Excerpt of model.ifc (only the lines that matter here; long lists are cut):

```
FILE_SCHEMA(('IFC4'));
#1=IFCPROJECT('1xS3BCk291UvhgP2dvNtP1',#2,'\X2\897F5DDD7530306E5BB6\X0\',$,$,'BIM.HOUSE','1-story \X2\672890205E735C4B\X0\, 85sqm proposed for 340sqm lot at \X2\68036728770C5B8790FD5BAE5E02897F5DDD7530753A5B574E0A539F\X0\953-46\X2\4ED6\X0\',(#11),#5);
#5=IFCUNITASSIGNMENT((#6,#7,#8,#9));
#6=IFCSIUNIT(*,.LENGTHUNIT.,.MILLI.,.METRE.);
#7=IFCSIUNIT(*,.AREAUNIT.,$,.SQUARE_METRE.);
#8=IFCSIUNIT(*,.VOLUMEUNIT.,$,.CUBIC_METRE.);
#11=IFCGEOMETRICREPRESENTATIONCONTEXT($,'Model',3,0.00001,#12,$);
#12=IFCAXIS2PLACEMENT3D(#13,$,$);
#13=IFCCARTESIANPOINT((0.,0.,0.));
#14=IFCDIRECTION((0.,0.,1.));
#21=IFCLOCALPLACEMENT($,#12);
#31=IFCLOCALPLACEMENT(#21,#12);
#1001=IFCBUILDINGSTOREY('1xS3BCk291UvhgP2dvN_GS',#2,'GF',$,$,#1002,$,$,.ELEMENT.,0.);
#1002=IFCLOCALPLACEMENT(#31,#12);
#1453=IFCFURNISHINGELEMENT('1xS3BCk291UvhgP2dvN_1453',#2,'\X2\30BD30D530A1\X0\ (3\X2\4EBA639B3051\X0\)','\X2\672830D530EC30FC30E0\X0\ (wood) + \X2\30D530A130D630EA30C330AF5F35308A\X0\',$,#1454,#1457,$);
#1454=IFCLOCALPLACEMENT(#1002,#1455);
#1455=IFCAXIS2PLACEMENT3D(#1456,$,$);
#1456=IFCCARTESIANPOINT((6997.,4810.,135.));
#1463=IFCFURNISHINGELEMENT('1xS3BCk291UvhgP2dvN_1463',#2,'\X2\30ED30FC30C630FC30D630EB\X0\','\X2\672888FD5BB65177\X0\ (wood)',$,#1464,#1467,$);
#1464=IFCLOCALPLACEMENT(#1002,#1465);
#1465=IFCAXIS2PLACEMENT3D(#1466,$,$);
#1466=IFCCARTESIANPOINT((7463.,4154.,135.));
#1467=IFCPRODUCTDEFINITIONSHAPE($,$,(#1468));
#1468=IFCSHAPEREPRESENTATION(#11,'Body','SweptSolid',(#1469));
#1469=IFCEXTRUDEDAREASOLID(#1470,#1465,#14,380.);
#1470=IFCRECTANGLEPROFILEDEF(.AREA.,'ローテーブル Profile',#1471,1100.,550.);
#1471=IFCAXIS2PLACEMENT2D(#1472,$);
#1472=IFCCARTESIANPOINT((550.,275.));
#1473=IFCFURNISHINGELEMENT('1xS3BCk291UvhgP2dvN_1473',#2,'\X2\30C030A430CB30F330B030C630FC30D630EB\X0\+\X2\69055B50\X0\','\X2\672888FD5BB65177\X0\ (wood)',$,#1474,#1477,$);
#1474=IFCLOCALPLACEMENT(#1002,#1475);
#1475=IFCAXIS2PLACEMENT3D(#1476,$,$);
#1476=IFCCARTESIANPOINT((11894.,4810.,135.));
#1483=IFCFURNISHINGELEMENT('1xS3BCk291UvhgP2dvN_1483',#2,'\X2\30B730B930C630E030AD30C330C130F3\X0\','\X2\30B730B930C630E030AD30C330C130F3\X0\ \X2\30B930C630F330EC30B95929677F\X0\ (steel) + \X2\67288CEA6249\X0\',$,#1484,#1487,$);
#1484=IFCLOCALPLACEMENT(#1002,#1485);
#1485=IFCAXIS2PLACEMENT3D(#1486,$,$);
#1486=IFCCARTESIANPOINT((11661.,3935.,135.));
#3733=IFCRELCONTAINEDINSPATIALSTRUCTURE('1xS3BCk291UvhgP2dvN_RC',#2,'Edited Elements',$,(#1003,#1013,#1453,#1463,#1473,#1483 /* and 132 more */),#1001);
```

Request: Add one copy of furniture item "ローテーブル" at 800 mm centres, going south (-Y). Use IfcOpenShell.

```python
import numpy as np
import ifcopenshell
import ifcopenshell.api.geometry
import ifcopenshell.api.root
import ifcopenshell.util.element
import ifcopenshell.util.placement
import ifcopenshell.util.unit

model = ifcopenshell.open("model.ifc")
unit_scale = ifcopenshell.util.unit.calculate_unit_scale(model)


def reuse_history(source, copy):
    """copy_class also copies each property set's owner history, people and application; keep the originals."""
    for rel in copy.IsDefinedBy:
        if rel.is_a("IfcRelDefinesByProperties") and (history := rel.RelatingPropertyDefinition.OwnerHistory):
            rel.RelatingPropertyDefinition.OwnerHistory = source.OwnerHistory
            ifcopenshell.util.element.remove_deep2(model, history)


source = model.by_guid("1xS3BCk291UvhgP2dvN_1463")
base = ifcopenshell.util.placement.get_local_placement(source.ObjectPlacement)
step = np.array([0.0, -1.0, 0.0]) * 0.8 / unit_scale

for i in range(1, 2):
    copy = ifcopenshell.api.root.copy_class(model, product=source)
    copy.Representation = ifcopenshell.util.element.copy_deep(
        model, source.Representation, exclude=["IfcGeometricRepresentationContext", "IfcRepresentationMap"]
    )
    reuse_history(source, copy)
    matrix = base.copy()
    matrix[:3, 3] += i * step
    print("added at", matrix[:3, 3].round(3) + 0.0)
    ifcopenshell.api.geometry.edit_object_placement(model, product=copy, matrix=matrix, is_si=False)

model.write("model-out.ifc")
```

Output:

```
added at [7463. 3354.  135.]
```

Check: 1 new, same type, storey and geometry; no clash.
